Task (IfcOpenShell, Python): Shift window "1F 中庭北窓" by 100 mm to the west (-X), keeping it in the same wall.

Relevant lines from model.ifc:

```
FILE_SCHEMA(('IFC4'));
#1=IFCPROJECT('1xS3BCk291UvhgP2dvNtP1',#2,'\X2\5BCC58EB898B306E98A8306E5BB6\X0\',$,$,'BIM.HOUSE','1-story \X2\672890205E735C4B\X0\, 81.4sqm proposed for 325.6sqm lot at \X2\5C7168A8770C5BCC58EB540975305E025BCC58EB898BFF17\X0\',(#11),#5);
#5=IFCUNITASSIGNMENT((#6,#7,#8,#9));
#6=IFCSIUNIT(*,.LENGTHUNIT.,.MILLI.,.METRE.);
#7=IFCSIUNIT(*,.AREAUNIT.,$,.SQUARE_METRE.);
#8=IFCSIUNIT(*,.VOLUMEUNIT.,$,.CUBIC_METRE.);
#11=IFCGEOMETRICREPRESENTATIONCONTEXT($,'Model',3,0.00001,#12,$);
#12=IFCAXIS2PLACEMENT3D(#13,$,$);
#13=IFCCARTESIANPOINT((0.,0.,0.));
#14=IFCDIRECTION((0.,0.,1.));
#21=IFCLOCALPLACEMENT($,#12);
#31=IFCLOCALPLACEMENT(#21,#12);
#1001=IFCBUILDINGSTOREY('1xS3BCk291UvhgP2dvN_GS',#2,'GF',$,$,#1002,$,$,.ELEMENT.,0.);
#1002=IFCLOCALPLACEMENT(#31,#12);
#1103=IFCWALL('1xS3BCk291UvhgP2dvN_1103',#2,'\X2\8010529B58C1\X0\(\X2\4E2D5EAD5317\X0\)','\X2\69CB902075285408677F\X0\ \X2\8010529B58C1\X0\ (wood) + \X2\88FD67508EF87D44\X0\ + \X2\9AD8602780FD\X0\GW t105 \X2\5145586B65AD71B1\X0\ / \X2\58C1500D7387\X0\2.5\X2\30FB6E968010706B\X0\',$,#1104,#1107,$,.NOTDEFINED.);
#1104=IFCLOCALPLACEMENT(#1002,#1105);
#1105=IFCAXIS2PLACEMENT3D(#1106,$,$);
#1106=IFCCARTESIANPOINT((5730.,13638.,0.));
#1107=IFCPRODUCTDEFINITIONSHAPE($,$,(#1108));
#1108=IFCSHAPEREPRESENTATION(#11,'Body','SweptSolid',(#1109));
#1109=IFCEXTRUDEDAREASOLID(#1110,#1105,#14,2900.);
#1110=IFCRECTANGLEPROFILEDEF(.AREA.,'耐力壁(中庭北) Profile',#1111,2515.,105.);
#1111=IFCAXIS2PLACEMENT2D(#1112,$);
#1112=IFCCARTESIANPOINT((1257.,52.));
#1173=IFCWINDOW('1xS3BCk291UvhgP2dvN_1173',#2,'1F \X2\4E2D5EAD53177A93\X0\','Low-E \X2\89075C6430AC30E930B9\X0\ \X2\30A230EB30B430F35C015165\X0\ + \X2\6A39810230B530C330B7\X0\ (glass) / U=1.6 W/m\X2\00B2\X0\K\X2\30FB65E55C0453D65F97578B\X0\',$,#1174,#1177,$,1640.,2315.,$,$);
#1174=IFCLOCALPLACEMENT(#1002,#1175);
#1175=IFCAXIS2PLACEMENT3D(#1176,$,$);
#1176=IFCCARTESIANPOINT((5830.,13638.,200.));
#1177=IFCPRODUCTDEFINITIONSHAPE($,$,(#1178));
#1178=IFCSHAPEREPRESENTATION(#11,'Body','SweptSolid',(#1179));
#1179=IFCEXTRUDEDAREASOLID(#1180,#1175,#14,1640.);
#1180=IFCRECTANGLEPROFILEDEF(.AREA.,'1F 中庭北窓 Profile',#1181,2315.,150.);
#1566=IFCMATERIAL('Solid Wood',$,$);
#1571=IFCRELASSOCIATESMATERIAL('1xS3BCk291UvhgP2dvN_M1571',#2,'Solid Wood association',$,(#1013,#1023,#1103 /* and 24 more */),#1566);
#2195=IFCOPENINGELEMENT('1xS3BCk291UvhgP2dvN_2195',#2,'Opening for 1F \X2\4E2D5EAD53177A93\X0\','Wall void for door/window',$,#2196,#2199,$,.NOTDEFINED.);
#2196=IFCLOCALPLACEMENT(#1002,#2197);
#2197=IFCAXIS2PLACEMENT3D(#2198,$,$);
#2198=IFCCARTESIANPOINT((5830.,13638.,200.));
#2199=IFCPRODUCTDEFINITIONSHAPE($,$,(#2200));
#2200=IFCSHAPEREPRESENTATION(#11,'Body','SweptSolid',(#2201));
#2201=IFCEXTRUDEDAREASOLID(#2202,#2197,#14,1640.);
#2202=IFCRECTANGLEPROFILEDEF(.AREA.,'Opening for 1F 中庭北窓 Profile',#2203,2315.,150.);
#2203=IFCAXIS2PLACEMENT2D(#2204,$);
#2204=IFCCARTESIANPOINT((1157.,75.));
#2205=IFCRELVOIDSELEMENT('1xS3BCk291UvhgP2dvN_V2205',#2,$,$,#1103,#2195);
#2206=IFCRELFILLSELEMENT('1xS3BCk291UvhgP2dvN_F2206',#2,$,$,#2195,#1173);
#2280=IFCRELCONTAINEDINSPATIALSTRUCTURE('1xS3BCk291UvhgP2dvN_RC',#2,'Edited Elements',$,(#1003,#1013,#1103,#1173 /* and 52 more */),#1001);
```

```python
import ifcopenshell
import ifcopenshell.api.geometry
import ifcopenshell.util.placement
import ifcopenshell.util.unit

model = ifcopenshell.open("model.ifc")
unit_scale = ifcopenshell.util.unit.calculate_unit_scale(model)

window = model.by_id(1173)
opening = window.FillsVoids[0].RelatingOpeningElement
wall = opening.VoidsElements[0].RelatingBuildingElement

wall_matrix = ifcopenshell.util.placement.get_local_placement(wall.ObjectPlacement)
shift = wall_matrix[:3, 0] * -0.1 / unit_scale
before = ifcopenshell.util.placement.get_local_placement(window.ObjectPlacement)[:3, 3].copy()

# The window is not placed relative to its opening, so move both.
for product in (opening, window):
    matrix = ifcopenshell.util.placement.get_local_placement(product.ObjectPlacement)
    matrix[:3, 3] += shift
    ifcopenshell.api.geometry.edit_object_placement(model, product=product, matrix=matrix, is_si=False)

after = ifcopenshell.util.placement.get_local_placement(window.ObjectPlacement)[:3, 3]
print("window moved by", (after - before).round(3) + 0.0)

model.write("model_edited.ifc")
```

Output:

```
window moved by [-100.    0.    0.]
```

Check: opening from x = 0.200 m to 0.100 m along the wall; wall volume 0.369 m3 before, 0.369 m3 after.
